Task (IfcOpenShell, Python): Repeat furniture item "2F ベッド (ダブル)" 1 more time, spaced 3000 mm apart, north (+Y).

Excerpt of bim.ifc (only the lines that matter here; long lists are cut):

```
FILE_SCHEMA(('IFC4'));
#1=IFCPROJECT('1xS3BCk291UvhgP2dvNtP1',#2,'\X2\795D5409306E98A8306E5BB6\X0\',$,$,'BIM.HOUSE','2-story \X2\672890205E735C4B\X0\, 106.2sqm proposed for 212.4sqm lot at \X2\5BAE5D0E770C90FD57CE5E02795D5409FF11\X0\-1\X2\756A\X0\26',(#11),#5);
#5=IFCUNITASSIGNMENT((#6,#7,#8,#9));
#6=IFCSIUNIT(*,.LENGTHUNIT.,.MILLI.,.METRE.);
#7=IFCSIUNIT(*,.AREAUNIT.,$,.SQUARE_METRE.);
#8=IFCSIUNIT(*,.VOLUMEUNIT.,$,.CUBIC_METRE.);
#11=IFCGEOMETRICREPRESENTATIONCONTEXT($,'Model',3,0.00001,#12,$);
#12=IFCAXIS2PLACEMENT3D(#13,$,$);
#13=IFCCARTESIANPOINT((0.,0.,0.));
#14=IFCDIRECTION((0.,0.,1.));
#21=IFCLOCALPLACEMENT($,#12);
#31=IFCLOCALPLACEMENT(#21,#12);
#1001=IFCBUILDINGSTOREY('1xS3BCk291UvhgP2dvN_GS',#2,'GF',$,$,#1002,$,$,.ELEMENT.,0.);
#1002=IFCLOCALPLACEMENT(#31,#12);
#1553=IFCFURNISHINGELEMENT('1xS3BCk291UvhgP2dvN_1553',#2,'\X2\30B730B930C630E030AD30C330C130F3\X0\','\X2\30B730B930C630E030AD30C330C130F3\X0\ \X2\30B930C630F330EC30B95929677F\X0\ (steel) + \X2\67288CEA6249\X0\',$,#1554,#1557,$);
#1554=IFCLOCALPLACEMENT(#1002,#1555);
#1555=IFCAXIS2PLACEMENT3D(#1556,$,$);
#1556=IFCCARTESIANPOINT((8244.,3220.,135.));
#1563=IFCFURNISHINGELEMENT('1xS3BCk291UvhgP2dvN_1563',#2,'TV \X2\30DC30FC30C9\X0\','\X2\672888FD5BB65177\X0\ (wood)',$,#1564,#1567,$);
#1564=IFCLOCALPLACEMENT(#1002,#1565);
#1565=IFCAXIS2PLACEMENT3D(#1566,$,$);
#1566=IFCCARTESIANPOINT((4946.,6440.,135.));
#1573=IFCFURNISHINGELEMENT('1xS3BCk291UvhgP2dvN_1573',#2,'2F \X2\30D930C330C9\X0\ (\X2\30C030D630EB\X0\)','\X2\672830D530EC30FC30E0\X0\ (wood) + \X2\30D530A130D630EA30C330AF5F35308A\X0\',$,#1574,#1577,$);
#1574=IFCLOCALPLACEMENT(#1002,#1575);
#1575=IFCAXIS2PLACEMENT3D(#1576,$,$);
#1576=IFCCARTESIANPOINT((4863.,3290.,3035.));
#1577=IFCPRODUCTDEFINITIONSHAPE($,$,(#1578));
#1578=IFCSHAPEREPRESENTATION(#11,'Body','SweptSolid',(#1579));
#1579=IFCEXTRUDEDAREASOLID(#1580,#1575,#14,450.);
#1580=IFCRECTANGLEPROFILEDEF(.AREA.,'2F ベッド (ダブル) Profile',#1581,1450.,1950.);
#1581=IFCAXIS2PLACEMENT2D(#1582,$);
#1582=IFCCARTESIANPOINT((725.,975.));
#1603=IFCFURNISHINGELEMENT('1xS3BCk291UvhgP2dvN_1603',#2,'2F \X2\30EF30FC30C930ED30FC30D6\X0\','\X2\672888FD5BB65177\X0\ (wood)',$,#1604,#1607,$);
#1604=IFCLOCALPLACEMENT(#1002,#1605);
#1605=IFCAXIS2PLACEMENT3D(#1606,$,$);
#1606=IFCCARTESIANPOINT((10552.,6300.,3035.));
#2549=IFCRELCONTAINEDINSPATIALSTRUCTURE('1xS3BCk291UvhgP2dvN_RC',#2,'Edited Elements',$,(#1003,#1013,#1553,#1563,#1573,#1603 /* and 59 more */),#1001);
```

```python
import numpy as np
import ifcopenshell
import ifcopenshell.api.geometry
import ifcopenshell.api.root
import ifcopenshell.util.element
import ifcopenshell.util.placement
import ifcopenshell.util.unit

model = ifcopenshell.open("bim.ifc")
unit_scale = ifcopenshell.util.unit.calculate_unit_scale(model)


def reuse_history(source, copy):
    """copy_class also copies each property set's owner history, people and application; keep the originals."""
    for rel in copy.IsDefinedBy:
        if rel.is_a("IfcRelDefinesByProperties") and (history := rel.RelatingPropertyDefinition.OwnerHistory):
            rel.RelatingPropertyDefinition.OwnerHistory = source.OwnerHistory
            ifcopenshell.util.element.remove_deep2(model, history)


source = model.by_id(1573)
base = ifcopenshell.util.placement.get_local_placement(source.ObjectPlacement)
step = np.array([0.0, 1.0, 0.0]) * 3 / unit_scale

for i in range(1, 2):
    copy = ifcopenshell.api.root.copy_class(model, product=source)
    copy.Representation = ifcopenshell.util.element.copy_deep(
        model, source.Representation, exclude=["IfcGeometricRepresentationContext", "IfcRepresentationMap"]
    )
    reuse_history(source, copy)
    matrix = base.copy()
    matrix[:3, 3] += i * step
    print("added at", matrix[:3, 3].round(3) + 0.0)
    ifcopenshell.api.geometry.edit_object_placement(model, product=copy, matrix=matrix, is_si=False)

model.write("bim_edited.ifc")
```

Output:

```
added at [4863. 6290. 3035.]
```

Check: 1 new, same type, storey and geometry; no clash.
